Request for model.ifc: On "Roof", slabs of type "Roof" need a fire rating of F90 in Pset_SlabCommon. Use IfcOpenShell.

First a look at what the model holds.

```python
import ifcopenshell
import ifcopenshell.util.element

model = ifcopenshell.open("model.ifc")
print(model.schema)
storey = next(s for s in model.by_type("IfcBuildingStorey") if s.Name == "Roof")
slabs = [e for e in ifcopenshell.util.element.get_decomposition(storey) if e.is_a("IfcSlab")]
seen = {}
for e in slabs:
    element_type = ifcopenshell.util.element.get_type(e)
    key = (element_type.Name if element_type != e and element_type else None, ifcopenshell.util.element.get_pset(e, "Pset_SlabCommon", "FireRating"))
    seen[key] = seen.get(key, 0) + 1
for (name, value), count in sorted(seen.items(), key=str):
    print(count, "x", name, "|", value)
```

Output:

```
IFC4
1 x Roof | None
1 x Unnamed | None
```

```python
import ifcopenshell
import ifcopenshell.api.pset
import ifcopenshell.util.element

model = ifcopenshell.open("model.ifc")

storey = next(s for s in model.by_type("IfcBuildingStorey") if s.Name == "Roof")
slabs = [e for e in ifcopenshell.util.element.get_decomposition(storey) if e.is_a("IfcSlab")]

count = 0
for e in slabs:
    element_type = ifcopenshell.util.element.get_type(e)
    if element_type in (None, e) or element_type.Name != "Roof":
        continue
    # add_pset returns the element's existing set when there is one.
    pset = ifcopenshell.api.pset.add_pset(model, product=e, name="Pset_SlabCommon")
    ifcopenshell.api.pset.edit_pset(model, pset=pset, properties={"FireRating": "F90"})
    count += 1

print(count, "slabs updated")

model.write("model_edited.ifc")
```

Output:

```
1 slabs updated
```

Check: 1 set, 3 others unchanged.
